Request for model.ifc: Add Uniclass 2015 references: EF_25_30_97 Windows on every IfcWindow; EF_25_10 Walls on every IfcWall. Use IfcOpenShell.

First a look at what the model holds.

```python
import ifcopenshell

model = ifcopenshell.open("model.ifc")
print(model.schema)
print("classifications:", [c.Name for c in model.by_type("IfcClassification")])
for ifc_class in ("IfcDoor", "IfcRoof", "IfcStair", "IfcWall", "IfcWindow"):
    print(ifc_class, len(model.by_type(ifc_class)))
```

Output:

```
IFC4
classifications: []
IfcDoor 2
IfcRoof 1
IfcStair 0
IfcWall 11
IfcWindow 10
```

```python
import ifcopenshell
import ifcopenshell.api.classification

model = ifcopenshell.open("model.ifc")

system = ifcopenshell.api.classification.add_classification(model, classification="Uniclass 2015")

codes = {
    "IfcWindow": ("EF_25_30_97", "Windows"),
    "IfcWall": ("EF_25_10", "Walls"),
}
for ifc_class, (code, name) in codes.items():
    products = model.by_type(ifc_class)
    ifcopenshell.api.classification.add_reference(
        model, products=products, classification=system, identification=code, name=name
    )
    print(code, len(products))

model.write("model-out.ifc")
```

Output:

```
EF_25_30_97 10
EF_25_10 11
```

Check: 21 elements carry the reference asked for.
